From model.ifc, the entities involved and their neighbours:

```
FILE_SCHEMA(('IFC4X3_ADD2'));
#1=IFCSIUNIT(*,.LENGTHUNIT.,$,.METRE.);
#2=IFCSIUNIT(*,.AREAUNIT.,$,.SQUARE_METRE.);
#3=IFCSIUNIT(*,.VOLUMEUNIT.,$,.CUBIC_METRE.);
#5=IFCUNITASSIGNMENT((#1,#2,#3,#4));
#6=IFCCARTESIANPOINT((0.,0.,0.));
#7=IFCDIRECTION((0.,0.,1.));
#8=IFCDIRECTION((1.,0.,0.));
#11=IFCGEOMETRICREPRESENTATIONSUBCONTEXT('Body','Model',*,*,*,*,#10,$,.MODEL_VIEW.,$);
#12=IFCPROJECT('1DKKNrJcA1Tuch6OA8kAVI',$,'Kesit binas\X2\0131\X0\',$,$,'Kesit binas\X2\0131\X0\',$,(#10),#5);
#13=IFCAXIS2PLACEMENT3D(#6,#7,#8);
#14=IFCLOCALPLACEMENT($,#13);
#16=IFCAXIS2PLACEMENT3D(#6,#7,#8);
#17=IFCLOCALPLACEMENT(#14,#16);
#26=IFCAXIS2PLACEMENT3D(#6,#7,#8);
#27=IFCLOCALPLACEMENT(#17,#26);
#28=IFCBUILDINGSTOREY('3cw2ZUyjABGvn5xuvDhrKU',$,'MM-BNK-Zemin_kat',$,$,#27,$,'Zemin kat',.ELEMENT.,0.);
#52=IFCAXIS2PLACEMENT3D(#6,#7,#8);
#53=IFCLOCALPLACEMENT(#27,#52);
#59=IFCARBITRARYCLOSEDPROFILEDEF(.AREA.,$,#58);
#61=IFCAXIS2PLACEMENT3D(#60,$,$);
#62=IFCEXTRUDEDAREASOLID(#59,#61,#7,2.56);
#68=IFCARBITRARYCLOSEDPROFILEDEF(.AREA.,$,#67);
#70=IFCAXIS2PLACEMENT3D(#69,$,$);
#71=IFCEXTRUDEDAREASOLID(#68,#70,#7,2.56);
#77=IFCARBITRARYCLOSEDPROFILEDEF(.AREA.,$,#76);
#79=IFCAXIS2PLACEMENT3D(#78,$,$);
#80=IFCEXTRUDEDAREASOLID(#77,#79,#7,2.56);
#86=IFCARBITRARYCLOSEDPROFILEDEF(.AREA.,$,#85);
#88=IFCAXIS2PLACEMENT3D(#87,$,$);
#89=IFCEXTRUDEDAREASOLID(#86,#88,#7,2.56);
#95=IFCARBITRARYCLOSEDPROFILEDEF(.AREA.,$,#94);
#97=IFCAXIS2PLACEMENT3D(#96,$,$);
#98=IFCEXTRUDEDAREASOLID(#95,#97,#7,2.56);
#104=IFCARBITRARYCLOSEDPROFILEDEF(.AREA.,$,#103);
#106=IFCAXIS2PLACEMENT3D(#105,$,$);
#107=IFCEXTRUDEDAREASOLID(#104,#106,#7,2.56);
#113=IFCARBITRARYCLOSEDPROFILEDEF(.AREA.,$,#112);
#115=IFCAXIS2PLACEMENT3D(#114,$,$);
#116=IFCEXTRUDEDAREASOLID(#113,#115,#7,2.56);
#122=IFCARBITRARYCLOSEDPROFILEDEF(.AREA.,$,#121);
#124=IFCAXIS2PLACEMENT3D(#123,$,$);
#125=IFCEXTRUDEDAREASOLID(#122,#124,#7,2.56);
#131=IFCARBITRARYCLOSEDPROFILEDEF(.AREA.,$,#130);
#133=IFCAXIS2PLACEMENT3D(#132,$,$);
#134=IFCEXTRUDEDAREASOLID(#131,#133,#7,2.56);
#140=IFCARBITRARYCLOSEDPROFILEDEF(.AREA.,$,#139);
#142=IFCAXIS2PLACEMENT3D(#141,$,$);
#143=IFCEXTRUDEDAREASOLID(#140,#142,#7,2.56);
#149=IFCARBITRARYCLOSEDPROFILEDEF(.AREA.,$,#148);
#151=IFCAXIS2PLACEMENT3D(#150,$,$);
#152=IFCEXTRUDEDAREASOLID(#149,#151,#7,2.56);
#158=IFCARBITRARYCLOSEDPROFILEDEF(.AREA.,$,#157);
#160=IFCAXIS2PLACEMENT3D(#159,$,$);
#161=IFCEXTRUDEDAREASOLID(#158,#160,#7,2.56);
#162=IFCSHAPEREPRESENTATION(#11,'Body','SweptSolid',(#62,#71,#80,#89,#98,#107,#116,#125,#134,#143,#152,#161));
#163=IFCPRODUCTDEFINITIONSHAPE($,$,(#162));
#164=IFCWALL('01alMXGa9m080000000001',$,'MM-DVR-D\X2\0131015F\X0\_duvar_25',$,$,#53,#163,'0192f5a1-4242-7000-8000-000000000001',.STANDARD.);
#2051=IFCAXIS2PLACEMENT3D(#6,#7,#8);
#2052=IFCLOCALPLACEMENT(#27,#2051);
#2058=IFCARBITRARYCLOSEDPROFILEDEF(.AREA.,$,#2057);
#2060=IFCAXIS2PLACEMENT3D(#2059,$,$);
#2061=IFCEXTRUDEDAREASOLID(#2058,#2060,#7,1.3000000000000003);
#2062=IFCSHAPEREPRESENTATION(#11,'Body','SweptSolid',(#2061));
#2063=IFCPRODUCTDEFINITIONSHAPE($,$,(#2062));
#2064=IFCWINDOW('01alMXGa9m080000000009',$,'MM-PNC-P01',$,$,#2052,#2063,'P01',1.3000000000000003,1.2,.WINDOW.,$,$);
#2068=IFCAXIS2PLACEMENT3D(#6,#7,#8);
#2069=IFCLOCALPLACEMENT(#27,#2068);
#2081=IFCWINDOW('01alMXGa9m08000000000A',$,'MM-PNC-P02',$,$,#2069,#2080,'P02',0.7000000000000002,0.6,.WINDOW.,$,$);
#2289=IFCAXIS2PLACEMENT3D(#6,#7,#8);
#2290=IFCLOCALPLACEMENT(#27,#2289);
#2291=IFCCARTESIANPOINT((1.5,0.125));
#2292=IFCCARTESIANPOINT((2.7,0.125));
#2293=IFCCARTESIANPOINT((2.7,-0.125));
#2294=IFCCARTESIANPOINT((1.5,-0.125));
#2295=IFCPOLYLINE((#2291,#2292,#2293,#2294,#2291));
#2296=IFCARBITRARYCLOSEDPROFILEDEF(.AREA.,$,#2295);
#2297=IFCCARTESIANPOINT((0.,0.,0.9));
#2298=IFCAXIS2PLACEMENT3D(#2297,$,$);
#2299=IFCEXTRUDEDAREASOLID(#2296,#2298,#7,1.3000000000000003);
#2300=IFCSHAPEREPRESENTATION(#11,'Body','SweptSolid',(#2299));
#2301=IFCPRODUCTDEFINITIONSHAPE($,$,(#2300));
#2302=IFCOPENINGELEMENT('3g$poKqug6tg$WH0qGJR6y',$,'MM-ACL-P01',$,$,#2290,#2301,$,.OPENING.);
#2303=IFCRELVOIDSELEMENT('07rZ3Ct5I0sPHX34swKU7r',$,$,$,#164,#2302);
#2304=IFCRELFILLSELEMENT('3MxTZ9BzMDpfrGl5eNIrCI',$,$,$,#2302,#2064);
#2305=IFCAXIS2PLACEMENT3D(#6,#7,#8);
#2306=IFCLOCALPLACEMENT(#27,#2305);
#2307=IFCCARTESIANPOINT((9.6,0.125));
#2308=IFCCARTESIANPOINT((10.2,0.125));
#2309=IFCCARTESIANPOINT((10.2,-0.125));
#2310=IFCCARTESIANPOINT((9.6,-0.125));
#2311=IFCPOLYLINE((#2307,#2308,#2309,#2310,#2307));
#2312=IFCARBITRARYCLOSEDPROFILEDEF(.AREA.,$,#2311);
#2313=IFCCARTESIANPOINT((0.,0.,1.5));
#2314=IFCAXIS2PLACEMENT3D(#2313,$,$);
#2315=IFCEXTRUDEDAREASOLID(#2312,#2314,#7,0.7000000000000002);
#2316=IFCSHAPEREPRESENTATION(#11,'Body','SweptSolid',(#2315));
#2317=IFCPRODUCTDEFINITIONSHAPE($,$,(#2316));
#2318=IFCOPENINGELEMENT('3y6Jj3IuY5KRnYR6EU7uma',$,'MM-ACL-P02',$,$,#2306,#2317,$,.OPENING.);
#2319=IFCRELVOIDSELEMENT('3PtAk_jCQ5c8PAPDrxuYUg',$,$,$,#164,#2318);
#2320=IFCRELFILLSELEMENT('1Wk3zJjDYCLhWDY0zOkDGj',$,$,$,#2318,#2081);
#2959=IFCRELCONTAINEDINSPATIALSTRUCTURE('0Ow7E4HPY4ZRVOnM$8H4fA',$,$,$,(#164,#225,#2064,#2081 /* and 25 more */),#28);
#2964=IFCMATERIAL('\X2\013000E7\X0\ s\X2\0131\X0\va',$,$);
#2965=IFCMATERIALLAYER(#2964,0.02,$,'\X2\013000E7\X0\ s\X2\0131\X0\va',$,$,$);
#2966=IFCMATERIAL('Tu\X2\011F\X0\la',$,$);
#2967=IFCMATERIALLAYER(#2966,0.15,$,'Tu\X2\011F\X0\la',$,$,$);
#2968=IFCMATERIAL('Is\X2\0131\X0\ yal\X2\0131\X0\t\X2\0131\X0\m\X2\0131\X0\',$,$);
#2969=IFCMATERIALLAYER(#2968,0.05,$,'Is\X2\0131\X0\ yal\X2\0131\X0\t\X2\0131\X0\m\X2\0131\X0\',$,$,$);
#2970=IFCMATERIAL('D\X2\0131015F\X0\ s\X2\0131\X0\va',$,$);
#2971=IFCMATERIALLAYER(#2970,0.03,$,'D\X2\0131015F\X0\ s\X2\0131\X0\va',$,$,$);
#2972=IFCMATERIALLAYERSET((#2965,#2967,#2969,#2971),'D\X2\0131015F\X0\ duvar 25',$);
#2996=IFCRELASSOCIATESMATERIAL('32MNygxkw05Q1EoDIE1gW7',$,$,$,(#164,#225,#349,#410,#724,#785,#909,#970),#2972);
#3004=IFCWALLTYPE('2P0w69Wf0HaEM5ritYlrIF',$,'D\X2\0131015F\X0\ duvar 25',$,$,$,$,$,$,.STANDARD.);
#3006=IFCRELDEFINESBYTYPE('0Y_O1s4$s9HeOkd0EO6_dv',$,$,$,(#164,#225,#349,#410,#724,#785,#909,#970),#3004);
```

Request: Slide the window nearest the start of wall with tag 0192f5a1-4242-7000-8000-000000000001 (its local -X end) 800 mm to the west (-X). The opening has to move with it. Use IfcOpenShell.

```python
import ifcopenshell
import ifcopenshell.api.geometry
import ifcopenshell.util.placement
import ifcopenshell.util.unit

model = ifcopenshell.open("model.ifc")
unit_scale = ifcopenshell.util.unit.calculate_unit_scale(model)

window = model.by_guid("01alMXGa9m080000000009")
opening = window.FillsVoids[0].RelatingOpeningElement
wall = opening.VoidsElements[0].RelatingBuildingElement

wall_matrix = ifcopenshell.util.placement.get_local_placement(wall.ObjectPlacement)
shift = wall_matrix[:3, 0] * -0.8 / unit_scale
before = ifcopenshell.util.placement.get_local_placement(window.ObjectPlacement)[:3, 3].copy()

# The window is not placed relative to its opening, so move both.
for product in (opening, window):
    matrix = ifcopenshell.util.placement.get_local_placement(product.ObjectPlacement)
    matrix[:3, 3] += shift
    ifcopenshell.api.geometry.edit_object_placement(model, product=product, matrix=matrix, is_si=False)

after = ifcopenshell.util.placement.get_local_placement(window.ObjectPlacement)[:3, 3]
print("window moved by", (after - before).round(3) + 0.0)

model.write("model_rev.ifc")
```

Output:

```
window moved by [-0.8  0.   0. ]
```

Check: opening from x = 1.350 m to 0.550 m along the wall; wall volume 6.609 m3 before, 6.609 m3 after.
